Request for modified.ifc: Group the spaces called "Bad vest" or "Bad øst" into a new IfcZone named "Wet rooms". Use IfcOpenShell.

First a look at what the model holds.

```python
import ifcopenshell

model = ifcopenshell.open("modified.ifc")
print(model.schema)
seen = {}
for space in model.by_type("IfcSpace"):
    seen[space.LongName] = seen.get(space.LongName, 0) + 1
for name, count in sorted(seen.items(), key=str):
    print(count, "x", name)
print("zones:", [z.Name for z in model.by_type("IfcZone")][:20])
```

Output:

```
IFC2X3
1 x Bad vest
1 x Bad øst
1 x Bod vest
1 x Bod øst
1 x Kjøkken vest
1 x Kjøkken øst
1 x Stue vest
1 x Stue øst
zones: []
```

```python
import ifcopenshell
import ifcopenshell.api.group
import ifcopenshell.api.root

model = ifcopenshell.open("modified.ifc")

names = {"Bad vest", "Bad øst"}
spaces = [s for s in model.by_type("IfcSpace") if s.LongName in names]

zone = ifcopenshell.api.root.create_entity(model, ifc_class="IfcZone", name="Wet rooms")
ifcopenshell.api.group.assign_group(model, products=spaces, group=zone)
print(len(spaces), "spaces in", zone.Name)

model.write("modified_edited.ifc")
```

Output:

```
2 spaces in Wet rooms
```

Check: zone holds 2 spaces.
